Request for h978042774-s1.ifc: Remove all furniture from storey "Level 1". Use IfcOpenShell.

First a look at what the model holds.

```python
import ifcopenshell
import ifcopenshell.util.element

model = ifcopenshell.open("h978042774-s1.ifc")
print(model.schema)
storey = next(s for s in model.by_type("IfcBuildingStorey") if s.Name == "Level 1")
furniture = [e for e in ifcopenshell.util.element.get_decomposition(storey) if e.is_a("IfcFurnishingElement")]
seen = {}
for e in furniture:
    element_type = ifcopenshell.util.element.get_type(e)
    name = element_type.Name if element_type not in (None, e) else None
    seen[name] = seen.get(name, 0) + 1
for name, count in sorted(seen.items(), key=str):
    print(count, "x", name)
```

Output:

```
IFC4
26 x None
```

```python
import ifcopenshell
import ifcopenshell.api.root
import ifcopenshell.util.element

model = ifcopenshell.open("h978042774-s1.ifc")

storey = next(s for s in model.by_type("IfcBuildingStorey") if s.Name == "Level 1")
furniture = [e for e in ifcopenshell.util.element.get_decomposition(storey) if e.is_a("IfcFurnishingElement")]

for e in furniture:
    ifcopenshell.api.root.remove_product(model, product=e)
print(len(furniture), "removed")

model.write("h978042774-s1-out.ifc")
```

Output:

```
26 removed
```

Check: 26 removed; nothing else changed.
